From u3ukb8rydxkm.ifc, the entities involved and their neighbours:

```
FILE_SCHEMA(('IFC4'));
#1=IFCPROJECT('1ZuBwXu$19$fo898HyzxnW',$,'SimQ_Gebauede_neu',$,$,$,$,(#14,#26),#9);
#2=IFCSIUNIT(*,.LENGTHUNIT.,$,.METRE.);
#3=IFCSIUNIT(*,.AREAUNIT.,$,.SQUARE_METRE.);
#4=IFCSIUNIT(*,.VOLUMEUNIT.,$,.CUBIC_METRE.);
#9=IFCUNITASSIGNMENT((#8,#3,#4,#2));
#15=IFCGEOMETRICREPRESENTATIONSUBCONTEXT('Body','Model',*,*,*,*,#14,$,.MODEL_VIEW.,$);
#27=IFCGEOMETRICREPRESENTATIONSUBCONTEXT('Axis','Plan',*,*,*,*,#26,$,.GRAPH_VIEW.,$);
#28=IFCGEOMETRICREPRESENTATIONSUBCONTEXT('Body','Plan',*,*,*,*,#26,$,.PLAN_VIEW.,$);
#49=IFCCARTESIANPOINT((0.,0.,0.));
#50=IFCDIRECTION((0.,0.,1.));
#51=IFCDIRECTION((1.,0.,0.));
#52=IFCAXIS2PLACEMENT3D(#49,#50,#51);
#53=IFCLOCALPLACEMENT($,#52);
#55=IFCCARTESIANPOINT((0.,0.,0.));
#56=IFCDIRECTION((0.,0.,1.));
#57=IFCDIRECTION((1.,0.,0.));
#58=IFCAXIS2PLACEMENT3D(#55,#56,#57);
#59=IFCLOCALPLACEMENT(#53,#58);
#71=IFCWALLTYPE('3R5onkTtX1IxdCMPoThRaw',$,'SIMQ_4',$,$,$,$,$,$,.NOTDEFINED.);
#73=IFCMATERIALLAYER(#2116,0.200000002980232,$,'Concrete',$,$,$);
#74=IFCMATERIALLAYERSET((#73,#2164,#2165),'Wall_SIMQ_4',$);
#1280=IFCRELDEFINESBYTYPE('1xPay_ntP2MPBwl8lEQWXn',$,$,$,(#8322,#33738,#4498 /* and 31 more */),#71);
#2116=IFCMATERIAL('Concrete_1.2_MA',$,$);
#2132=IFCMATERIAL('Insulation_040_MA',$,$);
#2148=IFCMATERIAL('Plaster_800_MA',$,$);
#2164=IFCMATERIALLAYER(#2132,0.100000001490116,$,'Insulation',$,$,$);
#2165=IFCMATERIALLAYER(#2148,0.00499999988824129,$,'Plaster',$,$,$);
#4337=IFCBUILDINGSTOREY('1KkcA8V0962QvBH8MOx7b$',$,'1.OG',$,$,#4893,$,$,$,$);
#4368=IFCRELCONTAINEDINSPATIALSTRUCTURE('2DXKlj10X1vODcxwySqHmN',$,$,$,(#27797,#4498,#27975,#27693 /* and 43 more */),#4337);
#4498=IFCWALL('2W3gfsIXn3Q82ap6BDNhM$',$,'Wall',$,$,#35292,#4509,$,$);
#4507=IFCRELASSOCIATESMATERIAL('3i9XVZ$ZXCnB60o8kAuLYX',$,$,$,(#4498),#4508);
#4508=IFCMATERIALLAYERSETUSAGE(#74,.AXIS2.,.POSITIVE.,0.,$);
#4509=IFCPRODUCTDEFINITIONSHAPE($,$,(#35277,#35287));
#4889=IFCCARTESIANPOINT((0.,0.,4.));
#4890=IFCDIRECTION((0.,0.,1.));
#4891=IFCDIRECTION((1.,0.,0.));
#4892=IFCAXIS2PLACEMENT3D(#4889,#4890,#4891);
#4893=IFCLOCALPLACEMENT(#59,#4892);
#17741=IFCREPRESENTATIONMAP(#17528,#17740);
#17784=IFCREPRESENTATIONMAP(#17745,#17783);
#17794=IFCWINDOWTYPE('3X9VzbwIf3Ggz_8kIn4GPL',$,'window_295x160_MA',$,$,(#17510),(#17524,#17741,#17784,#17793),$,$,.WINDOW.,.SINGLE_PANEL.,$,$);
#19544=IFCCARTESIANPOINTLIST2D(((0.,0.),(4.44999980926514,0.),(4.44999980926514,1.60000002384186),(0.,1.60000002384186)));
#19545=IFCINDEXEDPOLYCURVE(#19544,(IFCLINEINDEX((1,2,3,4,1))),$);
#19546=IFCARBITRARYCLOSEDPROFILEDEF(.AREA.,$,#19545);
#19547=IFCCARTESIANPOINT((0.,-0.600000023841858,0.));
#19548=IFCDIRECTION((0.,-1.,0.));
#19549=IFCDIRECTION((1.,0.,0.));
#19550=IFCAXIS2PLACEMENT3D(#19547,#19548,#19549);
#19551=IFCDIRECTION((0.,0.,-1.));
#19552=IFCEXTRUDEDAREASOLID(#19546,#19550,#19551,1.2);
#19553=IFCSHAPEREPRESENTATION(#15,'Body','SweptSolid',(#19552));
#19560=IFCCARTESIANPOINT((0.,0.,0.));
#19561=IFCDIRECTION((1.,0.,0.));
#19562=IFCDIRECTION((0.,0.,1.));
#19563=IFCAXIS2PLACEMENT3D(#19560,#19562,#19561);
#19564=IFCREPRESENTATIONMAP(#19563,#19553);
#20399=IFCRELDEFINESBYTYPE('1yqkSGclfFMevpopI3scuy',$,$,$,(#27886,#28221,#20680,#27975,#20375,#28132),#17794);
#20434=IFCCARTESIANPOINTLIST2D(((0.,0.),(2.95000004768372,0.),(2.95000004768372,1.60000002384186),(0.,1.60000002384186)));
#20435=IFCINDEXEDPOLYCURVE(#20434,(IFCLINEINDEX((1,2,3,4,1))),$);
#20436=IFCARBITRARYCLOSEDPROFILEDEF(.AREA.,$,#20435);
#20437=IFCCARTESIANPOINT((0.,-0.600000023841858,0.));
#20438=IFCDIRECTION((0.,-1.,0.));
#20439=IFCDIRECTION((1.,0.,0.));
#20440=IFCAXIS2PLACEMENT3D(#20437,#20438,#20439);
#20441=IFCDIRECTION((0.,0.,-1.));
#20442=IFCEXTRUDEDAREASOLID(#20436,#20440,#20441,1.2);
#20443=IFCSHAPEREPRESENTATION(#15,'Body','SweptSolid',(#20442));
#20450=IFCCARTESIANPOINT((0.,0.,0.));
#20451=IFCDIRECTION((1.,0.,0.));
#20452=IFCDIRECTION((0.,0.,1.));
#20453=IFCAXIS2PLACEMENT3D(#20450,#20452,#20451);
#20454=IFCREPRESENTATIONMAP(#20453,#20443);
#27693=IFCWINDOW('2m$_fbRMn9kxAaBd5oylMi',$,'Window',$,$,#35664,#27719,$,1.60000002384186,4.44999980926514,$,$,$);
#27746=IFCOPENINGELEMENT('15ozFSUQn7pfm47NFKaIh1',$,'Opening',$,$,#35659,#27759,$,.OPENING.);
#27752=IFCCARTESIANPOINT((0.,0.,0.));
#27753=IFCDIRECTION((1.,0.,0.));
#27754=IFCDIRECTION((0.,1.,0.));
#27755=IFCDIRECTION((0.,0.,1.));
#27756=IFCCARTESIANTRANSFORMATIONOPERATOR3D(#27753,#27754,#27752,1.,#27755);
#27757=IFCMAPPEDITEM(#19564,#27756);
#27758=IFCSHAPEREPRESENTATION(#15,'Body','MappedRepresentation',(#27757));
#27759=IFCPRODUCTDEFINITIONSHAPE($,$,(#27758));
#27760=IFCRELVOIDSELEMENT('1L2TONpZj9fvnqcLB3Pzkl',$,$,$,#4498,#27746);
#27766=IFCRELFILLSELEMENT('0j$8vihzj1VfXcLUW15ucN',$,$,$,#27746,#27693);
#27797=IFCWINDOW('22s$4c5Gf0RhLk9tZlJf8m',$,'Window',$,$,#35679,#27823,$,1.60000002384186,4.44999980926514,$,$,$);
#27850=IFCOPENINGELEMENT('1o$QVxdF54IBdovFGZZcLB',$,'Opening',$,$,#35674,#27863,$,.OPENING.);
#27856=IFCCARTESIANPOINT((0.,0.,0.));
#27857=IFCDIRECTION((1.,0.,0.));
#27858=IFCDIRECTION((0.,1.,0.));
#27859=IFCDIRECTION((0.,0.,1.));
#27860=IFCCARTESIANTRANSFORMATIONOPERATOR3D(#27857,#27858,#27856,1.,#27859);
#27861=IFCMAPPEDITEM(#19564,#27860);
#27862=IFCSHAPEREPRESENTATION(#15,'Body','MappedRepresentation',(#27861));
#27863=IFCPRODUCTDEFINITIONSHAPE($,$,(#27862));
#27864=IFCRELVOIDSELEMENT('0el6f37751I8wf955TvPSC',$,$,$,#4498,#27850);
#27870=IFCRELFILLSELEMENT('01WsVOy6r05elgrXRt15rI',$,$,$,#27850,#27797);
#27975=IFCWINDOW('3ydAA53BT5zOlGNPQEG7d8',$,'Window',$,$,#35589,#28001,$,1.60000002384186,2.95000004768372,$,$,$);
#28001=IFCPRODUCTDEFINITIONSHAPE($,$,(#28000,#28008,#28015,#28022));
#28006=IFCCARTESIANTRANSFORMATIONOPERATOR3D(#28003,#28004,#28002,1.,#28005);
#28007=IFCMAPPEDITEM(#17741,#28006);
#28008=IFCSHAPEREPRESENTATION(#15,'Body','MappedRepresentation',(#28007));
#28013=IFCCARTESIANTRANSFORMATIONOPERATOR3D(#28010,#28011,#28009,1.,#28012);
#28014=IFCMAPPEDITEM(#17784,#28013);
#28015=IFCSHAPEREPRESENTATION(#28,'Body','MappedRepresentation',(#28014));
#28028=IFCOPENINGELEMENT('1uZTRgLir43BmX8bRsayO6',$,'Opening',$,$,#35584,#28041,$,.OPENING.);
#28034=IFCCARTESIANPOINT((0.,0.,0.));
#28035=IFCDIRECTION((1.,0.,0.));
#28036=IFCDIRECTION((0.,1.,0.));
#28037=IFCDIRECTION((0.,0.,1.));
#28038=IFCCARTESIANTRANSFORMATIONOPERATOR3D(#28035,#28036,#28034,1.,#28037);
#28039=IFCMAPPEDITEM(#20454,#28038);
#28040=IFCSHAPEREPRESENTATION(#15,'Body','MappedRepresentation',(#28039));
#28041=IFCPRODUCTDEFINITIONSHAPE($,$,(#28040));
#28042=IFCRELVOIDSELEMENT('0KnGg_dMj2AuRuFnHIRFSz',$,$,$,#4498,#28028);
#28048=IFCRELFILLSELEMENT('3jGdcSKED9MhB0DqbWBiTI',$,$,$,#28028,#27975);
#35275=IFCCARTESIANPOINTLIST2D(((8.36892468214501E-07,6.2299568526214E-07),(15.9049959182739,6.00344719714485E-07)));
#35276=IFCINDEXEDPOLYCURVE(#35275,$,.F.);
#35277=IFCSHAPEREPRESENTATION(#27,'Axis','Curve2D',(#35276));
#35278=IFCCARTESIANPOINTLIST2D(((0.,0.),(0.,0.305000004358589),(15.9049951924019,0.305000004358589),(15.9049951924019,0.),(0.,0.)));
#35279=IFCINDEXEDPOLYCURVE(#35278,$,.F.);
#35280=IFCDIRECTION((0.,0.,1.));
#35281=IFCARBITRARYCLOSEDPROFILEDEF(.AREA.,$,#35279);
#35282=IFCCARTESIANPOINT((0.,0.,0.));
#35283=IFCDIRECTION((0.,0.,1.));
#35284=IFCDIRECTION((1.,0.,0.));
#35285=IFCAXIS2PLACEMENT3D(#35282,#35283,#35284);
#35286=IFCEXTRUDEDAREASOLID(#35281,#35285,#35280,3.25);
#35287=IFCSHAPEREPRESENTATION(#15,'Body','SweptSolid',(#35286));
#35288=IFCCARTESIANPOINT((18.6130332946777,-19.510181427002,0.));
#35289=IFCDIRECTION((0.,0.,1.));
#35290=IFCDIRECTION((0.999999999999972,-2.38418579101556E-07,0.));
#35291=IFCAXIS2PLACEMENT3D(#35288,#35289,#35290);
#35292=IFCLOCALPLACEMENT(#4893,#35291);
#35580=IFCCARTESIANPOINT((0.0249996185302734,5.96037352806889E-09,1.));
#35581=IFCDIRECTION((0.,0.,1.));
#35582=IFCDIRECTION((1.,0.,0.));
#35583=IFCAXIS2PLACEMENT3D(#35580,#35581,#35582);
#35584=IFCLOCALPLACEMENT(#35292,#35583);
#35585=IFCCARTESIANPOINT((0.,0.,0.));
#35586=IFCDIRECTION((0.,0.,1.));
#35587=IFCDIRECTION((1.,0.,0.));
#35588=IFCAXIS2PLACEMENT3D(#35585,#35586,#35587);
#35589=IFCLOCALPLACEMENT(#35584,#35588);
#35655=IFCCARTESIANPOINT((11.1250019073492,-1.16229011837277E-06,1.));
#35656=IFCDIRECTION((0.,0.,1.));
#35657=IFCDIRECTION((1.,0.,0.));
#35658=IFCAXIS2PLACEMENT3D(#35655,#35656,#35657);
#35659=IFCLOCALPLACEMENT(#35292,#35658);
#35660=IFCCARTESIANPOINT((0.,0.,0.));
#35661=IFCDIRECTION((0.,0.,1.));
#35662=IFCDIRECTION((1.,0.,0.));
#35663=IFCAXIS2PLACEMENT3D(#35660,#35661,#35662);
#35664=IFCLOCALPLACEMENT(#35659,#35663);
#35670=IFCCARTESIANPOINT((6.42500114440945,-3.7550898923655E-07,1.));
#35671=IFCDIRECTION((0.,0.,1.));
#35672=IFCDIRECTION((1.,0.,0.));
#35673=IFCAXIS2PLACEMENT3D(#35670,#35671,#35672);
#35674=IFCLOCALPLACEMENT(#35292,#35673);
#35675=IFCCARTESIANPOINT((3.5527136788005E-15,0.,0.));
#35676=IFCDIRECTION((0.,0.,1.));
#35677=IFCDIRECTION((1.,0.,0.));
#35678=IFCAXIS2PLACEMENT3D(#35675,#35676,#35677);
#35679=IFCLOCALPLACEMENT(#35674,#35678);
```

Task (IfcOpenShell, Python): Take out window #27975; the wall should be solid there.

```python
import ifcopenshell
import ifcopenshell.api.feature
import ifcopenshell.api.root
import ifcopenshell.geom
import ifcopenshell.util.shape

model = ifcopenshell.open("u3ukb8rydxkm.ifc")
settings = ifcopenshell.geom.settings()


def volume(element):
    """Net volume in cubic metres, openings subtracted."""
    shape = ifcopenshell.geom.create_shape(settings, element)
    return ifcopenshell.util.shape.get_volume(shape.geometry)


window = model.by_id(27975)
opening = window.FillsVoids[0].RelatingOpeningElement
wall = opening.VoidsElements[0].RelatingBuildingElement
before = volume(wall)

ifcopenshell.api.root.remove_product(model, product=window)
ifcopenshell.api.feature.remove_feature(model, feature=opening)

after = volume(wall)

print(f"wall volume {before:.3f} -> {after:.3f} m3")

model.write("u3ukb8rydxkm_updated.ifc")
```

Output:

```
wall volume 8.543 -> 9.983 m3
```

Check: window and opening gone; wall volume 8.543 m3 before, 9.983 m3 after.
